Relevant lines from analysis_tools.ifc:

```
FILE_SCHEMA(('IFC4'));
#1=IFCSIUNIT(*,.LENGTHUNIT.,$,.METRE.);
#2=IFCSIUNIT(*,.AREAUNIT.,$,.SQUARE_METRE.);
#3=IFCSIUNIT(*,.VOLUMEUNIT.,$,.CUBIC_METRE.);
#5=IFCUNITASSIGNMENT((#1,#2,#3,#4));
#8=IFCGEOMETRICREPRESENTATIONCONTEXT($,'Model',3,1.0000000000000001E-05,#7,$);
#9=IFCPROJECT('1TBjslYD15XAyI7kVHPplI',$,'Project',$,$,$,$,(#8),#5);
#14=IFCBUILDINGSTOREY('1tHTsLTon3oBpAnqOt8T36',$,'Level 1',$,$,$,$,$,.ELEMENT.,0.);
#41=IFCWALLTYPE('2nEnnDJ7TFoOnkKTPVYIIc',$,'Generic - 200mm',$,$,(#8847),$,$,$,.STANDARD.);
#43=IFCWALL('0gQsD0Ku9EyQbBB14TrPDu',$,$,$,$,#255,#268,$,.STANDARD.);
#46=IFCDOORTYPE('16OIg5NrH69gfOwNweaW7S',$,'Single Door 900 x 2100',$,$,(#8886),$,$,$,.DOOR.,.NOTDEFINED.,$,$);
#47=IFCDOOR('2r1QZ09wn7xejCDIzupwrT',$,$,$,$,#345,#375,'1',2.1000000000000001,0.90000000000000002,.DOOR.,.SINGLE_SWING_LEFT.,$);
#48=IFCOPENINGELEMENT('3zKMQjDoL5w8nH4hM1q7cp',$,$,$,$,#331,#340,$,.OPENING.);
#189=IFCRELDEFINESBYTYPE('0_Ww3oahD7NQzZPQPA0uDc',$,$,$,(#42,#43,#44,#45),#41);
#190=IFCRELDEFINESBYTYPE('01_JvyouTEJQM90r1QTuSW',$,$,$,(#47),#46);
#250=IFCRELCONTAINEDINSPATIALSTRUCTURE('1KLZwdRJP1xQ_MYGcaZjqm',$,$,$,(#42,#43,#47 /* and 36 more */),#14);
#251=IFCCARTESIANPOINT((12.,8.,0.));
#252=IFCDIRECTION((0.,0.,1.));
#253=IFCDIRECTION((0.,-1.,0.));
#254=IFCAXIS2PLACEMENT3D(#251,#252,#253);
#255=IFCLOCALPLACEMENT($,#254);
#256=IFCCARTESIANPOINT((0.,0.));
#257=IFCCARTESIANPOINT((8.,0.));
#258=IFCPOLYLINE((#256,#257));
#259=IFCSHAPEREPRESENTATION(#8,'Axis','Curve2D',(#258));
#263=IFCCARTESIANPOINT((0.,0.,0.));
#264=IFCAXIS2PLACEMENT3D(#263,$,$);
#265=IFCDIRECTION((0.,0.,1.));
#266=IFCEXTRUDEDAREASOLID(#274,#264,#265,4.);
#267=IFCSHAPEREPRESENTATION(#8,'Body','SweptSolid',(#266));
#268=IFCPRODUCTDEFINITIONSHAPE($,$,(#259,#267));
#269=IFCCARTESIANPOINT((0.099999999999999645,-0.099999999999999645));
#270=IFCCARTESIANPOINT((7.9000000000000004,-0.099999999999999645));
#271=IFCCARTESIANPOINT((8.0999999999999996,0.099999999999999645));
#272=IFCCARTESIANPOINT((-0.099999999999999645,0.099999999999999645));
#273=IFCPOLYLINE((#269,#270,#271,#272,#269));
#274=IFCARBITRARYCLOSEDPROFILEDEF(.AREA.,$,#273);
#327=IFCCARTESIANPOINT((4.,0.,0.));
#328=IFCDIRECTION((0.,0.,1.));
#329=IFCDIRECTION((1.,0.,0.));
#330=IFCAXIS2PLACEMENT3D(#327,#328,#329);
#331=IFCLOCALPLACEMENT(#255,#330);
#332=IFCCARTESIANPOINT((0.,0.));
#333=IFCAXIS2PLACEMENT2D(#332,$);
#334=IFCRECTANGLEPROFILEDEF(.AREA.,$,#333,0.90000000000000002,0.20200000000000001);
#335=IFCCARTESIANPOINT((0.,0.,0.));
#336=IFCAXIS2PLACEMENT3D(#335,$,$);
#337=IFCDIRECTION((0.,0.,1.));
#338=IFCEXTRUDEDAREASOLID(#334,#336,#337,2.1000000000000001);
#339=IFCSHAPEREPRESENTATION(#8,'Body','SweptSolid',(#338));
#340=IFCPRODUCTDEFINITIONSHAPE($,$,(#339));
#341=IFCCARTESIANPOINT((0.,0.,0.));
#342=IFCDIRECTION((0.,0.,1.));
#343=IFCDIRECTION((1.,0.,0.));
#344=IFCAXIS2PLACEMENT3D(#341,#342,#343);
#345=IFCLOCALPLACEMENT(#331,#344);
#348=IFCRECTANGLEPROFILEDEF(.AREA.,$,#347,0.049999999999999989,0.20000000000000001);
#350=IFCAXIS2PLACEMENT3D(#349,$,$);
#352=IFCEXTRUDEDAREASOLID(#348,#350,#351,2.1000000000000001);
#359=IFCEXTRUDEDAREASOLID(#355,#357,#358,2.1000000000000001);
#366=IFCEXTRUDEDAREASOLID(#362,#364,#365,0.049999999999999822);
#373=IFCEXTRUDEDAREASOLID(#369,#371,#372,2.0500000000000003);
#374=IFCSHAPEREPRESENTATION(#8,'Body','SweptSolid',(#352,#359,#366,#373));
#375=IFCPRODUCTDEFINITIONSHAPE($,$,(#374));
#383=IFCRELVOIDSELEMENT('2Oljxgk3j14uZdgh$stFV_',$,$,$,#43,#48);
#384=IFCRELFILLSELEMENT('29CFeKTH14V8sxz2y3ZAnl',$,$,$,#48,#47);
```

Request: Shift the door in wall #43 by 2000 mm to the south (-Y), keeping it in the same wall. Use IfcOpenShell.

```python
import ifcopenshell
import ifcopenshell.api.geometry
import ifcopenshell.util.placement
import ifcopenshell.util.unit

model = ifcopenshell.open("analysis_tools.ifc")
unit_scale = ifcopenshell.util.unit.calculate_unit_scale(model)

door = model.by_guid("2r1QZ09wn7xejCDIzupwrT")
opening = door.FillsVoids[0].RelatingOpeningElement
wall = opening.VoidsElements[0].RelatingBuildingElement

wall_matrix = ifcopenshell.util.placement.get_local_placement(wall.ObjectPlacement)
shift = wall_matrix[:3, 0] * 2 / unit_scale
before = ifcopenshell.util.placement.get_local_placement(door.ObjectPlacement)[:3, 3].copy()

# The door is placed relative to its opening, so it follows when the opening moves.
matrix = ifcopenshell.util.placement.get_local_placement(opening.ObjectPlacement)
matrix[:3, 3] += shift
ifcopenshell.api.geometry.edit_object_placement(
    model, product=opening, matrix=matrix, is_si=False, should_transform_children=True
)

after = ifcopenshell.util.placement.get_local_placement(door.ObjectPlacement)[:3, 3]
print("door moved by", (after - before).round(3) + 0.0)

model.write("analysis_tools_v2.ifc")
```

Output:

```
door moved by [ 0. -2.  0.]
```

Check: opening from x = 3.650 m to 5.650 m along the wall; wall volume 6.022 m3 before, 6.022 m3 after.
